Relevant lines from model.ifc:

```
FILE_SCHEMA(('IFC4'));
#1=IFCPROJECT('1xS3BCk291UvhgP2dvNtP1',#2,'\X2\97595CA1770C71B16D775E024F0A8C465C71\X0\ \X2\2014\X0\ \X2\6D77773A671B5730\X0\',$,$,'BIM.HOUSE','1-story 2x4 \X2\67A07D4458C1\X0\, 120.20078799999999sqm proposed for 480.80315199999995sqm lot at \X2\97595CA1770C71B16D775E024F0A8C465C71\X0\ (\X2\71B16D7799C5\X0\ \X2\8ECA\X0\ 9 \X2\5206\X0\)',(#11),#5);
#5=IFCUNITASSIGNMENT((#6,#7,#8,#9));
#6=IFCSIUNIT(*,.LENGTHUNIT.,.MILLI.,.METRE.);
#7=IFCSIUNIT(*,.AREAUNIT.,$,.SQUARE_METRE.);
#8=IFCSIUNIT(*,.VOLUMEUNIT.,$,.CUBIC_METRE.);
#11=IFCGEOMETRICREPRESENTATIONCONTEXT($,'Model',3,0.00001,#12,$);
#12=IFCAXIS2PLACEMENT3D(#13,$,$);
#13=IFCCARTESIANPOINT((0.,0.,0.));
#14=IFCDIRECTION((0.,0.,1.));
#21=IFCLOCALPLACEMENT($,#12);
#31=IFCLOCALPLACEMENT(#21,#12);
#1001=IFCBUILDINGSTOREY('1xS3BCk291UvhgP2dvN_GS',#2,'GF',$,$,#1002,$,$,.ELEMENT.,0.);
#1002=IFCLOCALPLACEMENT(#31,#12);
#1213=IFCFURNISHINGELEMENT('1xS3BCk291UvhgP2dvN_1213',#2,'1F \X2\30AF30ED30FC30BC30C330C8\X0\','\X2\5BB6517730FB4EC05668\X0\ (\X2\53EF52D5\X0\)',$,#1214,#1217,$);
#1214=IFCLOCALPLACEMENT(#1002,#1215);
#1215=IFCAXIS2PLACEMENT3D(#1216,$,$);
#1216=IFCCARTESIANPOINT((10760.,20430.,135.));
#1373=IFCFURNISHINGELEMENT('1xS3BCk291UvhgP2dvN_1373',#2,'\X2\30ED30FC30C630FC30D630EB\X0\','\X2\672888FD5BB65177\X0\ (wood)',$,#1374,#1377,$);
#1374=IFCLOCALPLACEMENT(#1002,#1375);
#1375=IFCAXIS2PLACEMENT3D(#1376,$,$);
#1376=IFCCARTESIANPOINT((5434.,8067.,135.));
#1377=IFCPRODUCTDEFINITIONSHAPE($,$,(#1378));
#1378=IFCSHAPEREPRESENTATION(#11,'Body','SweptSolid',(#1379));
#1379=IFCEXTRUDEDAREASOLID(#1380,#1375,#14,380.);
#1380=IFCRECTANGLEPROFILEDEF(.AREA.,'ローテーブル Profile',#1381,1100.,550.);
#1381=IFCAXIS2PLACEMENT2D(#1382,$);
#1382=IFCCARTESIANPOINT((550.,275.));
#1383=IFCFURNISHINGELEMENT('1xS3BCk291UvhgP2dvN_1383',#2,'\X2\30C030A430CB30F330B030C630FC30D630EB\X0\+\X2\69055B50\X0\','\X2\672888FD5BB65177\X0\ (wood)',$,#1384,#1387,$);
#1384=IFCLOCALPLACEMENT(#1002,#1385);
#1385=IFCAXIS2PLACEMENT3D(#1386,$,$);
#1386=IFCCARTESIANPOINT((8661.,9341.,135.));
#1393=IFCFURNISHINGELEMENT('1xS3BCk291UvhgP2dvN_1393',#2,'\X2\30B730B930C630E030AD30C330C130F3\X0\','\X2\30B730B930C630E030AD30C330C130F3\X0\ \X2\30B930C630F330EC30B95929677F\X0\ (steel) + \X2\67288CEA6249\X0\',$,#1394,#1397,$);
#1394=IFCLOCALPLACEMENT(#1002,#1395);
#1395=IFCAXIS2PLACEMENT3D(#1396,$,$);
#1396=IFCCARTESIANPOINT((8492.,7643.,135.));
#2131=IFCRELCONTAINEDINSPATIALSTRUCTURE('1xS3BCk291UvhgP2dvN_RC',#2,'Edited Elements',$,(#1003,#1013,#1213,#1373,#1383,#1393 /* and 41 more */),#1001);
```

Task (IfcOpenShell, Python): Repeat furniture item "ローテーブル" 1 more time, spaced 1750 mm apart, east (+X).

```python
import numpy as np
import ifcopenshell
import ifcopenshell.api.geometry
import ifcopenshell.api.root
import ifcopenshell.util.element
import ifcopenshell.util.placement
import ifcopenshell.util.unit

model = ifcopenshell.open("model.ifc")
unit_scale = ifcopenshell.util.unit.calculate_unit_scale(model)


def reuse_history(source, copy):
    """copy_class also copies each property set's owner history, people and application; keep the originals."""
    for rel in copy.IsDefinedBy:
        if rel.is_a("IfcRelDefinesByProperties") and (history := rel.RelatingPropertyDefinition.OwnerHistory):
            rel.RelatingPropertyDefinition.OwnerHistory = source.OwnerHistory
            ifcopenshell.util.element.remove_deep2(model, history)


source = model.by_id(1373)
base = ifcopenshell.util.placement.get_local_placement(source.ObjectPlacement)
step = np.array([1.0, 0.0, 0.0]) * 1.75 / unit_scale

for i in range(1, 2):
    copy = ifcopenshell.api.root.copy_class(model, product=source)
    copy.Representation = ifcopenshell.util.element.copy_deep(
        model, source.Representation, exclude=["IfcGeometricRepresentationContext", "IfcRepresentationMap"]
    )
    reuse_history(source, copy)
    matrix = base.copy()
    matrix[:3, 3] += i * step
    print("added at", matrix[:3, 3].round(3) + 0.0)
    ifcopenshell.api.geometry.edit_object_placement(model, product=copy, matrix=matrix, is_si=False)

model.write("model-out.ifc")
```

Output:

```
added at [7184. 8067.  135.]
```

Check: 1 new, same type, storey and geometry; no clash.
